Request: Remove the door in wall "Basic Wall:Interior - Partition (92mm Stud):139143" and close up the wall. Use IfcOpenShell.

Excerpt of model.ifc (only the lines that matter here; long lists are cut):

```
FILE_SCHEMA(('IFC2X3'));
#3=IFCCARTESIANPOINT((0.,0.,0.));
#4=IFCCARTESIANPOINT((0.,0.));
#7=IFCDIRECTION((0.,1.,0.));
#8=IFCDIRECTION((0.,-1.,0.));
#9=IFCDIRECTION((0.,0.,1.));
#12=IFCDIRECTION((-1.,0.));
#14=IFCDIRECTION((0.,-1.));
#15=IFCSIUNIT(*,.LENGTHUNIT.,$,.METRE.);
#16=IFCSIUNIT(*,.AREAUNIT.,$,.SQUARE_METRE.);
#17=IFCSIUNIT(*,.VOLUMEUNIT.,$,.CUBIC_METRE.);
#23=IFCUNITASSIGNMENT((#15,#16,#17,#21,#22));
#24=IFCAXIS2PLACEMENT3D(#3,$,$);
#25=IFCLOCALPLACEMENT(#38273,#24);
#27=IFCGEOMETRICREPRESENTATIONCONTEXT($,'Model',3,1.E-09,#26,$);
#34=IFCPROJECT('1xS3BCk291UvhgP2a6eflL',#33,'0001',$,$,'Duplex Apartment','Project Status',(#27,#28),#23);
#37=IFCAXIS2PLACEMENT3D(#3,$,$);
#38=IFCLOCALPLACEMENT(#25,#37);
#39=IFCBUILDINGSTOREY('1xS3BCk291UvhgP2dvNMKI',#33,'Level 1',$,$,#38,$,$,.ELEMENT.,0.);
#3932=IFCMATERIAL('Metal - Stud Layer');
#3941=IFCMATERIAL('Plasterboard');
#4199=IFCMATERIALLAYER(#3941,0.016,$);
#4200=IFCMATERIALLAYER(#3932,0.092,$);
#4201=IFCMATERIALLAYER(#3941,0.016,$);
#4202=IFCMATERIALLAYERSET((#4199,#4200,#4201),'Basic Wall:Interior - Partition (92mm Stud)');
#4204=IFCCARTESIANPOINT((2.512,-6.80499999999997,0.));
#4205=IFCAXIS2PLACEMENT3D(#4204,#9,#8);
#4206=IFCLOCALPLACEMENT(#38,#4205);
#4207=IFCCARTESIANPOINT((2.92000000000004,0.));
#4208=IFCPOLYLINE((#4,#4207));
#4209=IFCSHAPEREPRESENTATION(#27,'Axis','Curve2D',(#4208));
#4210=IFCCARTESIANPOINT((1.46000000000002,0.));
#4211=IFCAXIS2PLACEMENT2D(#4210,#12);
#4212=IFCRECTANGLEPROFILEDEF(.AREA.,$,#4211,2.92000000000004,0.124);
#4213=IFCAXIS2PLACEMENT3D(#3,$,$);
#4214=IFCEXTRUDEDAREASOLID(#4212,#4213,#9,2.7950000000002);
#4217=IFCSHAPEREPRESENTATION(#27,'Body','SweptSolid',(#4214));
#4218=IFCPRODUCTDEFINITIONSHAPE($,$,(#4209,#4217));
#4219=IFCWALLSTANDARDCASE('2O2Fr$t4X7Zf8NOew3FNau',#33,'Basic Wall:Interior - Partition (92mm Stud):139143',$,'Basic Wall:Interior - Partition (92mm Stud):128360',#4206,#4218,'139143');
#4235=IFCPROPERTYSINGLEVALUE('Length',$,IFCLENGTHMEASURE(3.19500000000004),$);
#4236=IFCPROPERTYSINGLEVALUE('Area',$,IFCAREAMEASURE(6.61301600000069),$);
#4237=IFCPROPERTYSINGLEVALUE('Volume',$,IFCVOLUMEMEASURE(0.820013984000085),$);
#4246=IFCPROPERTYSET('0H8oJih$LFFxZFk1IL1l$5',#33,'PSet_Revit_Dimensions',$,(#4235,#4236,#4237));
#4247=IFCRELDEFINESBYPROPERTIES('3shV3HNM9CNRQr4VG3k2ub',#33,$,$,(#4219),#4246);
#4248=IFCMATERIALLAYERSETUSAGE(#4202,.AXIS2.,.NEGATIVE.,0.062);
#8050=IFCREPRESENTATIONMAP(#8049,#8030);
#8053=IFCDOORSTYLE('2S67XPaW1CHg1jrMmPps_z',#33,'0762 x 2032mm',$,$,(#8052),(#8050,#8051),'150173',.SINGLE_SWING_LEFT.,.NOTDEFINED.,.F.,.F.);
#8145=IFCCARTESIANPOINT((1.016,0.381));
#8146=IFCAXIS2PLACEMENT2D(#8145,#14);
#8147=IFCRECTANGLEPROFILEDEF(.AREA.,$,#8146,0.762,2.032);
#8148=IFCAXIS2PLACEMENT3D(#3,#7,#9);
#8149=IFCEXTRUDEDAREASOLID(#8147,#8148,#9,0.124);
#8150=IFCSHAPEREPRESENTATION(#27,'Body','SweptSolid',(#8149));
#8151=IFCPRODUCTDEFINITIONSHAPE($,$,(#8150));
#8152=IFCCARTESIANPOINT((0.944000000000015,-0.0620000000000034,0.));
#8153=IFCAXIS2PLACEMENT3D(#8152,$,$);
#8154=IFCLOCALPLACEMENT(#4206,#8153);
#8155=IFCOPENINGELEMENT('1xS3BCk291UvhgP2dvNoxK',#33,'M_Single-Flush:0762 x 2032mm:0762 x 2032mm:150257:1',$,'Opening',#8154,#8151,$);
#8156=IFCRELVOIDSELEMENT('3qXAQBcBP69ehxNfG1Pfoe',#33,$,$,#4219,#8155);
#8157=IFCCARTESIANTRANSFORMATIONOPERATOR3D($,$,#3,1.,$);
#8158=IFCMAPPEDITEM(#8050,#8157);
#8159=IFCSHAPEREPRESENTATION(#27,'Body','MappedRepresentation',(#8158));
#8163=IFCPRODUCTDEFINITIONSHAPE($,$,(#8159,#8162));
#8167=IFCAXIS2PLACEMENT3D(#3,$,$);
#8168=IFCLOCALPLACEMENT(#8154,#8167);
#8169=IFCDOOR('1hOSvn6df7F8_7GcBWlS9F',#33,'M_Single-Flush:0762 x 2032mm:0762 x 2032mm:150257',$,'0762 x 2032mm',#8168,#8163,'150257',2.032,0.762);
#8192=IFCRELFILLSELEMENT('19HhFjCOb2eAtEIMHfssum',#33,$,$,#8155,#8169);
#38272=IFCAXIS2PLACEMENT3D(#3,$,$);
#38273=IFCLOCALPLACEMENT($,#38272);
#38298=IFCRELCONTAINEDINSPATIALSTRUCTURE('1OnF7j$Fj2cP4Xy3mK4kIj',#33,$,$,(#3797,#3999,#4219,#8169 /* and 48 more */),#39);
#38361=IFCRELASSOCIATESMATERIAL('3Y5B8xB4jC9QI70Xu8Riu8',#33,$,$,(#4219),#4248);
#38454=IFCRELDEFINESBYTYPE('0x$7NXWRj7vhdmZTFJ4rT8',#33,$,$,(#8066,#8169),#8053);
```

```python
import ifcopenshell
import ifcopenshell.api.feature
import ifcopenshell.api.pset
import ifcopenshell.api.root
import ifcopenshell.geom
import ifcopenshell.util.element
import ifcopenshell.util.shape
import ifcopenshell.util.unit

model = ifcopenshell.open("model.ifc")
area_scale = ifcopenshell.util.unit.calculate_unit_scale(model, "AREAUNIT")
volume_scale = ifcopenshell.util.unit.calculate_unit_scale(model, "VOLUMEUNIT")
settings = ifcopenshell.geom.settings()


def volume(element):
    """Net volume in cubic metres, openings subtracted."""
    shape = ifcopenshell.geom.create_shape(settings, element)
    return ifcopenshell.util.shape.get_volume(shape.geometry)


door = model.by_guid("1hOSvn6df7F8_7GcBWlS9F")
opening = door.FillsVoids[0].RelatingOpeningElement
wall = opening.VoidsElements[0].RelatingBuildingElement
before = volume(wall)

ifcopenshell.api.root.remove_product(model, product=door)
ifcopenshell.api.feature.remove_feature(model, feature=opening)

after = volume(wall)
thickness = 0.124  # wall thickness in metres

# Update the wall's stored quantities.
pset = model.by_id(ifcopenshell.util.element.get_pset(wall, "PSet_Revit_Dimensions", should_inherit=False)["id"])
ifcopenshell.api.pset.edit_pset(model, pset=pset, properties={
    "Area": model.create_entity("IfcAreaMeasure", after / thickness / area_scale),
    "Volume": model.create_entity("IfcVolumeMeasure", after / volume_scale),
})

print(f"wall volume {before:.3f} -> {after:.3f} m3")

model.write("model_updated.ifc")
```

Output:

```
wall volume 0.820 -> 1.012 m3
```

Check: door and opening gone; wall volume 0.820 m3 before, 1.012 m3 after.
